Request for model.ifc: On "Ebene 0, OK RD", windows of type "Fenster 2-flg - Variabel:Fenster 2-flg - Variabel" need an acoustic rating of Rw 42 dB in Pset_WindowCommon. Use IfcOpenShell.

First a look at what the model holds.

```python
import ifcopenshell
import ifcopenshell.util.element

model = ifcopenshell.open("model.ifc")
print(model.schema)
storey = next(s for s in model.by_type("IfcBuildingStorey") if s.Name == "Ebene 0, OK RD")
windows = [e for e in ifcopenshell.util.element.get_decomposition(storey) if e.is_a("IfcWindow")]
seen = {}
for e in windows:
    element_type = ifcopenshell.util.element.get_type(e)
    key = (element_type.Name if element_type != e and element_type else None, ifcopenshell.util.element.get_pset(e, "Pset_WindowCommon", "AcousticRating"))
    seen[key] = seen.get(key, 0) + 1
for (name, value), count in sorted(seen.items(), key=str):
    print(count, "x", name, "|", value)
```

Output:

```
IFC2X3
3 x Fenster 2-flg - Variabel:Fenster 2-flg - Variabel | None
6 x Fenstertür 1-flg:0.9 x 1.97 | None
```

```python
import ifcopenshell
import ifcopenshell.api.pset
import ifcopenshell.util.element

model = ifcopenshell.open("model.ifc")

storey = next(s for s in model.by_type("IfcBuildingStorey") if s.Name == "Ebene 0, OK RD")
windows = [e for e in ifcopenshell.util.element.get_decomposition(storey) if e.is_a("IfcWindow")]

count = 0
for e in windows:
    element_type = ifcopenshell.util.element.get_type(e)
    if element_type in (None, e) or element_type.Name != "Fenster 2-flg - Variabel:Fenster 2-flg - Variabel":
        continue
    # add_pset returns the element's existing set when there is one.
    pset = ifcopenshell.api.pset.add_pset(model, product=e, name="Pset_WindowCommon")
    ifcopenshell.api.pset.edit_pset(model, pset=pset, properties={"AcousticRating": "Rw 42 dB"})
    count += 1

print(count, "windows updated")

model.write("model_updated.ifc")
```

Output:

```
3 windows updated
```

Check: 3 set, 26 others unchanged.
